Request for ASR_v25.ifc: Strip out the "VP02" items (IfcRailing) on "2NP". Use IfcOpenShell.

First a look at what the model holds.

```python
import ifcopenshell
import ifcopenshell.util.element

model = ifcopenshell.open("ASR_v25.ifc")
print(model.schema)
storey = next(s for s in model.by_type("IfcBuildingStorey") if s.Name == "2NP")
railings = [e for e in ifcopenshell.util.element.get_decomposition(storey) if e.is_a("IfcRailing")]
seen = {}
for e in railings:
    element_type = ifcopenshell.util.element.get_type(e)
    name = element_type.Name if element_type not in (None, e) else None
    seen[name] = seen.get(name, 0) + 1
for name, count in sorted(seen.items(), key=str):
    print(count, "x", name)
```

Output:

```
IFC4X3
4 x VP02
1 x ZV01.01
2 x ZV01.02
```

```python
import ifcopenshell
import ifcopenshell.api.root
import ifcopenshell.util.element

model = ifcopenshell.open("ASR_v25.ifc")

storey = next(s for s in model.by_type("IfcBuildingStorey") if s.Name == "2NP")
railings = [e for e in ifcopenshell.util.element.get_decomposition(storey) if e.is_a("IfcRailing")]
targets = [e for e in railings if (t := ifcopenshell.util.element.get_type(e)) not in (None, e) and t.Name == "VP02"]

for e in targets:
    ifcopenshell.api.root.remove_product(model, product=e)
print(len(targets), "removed")

model.write("ASR_v25_v2.ifc")
```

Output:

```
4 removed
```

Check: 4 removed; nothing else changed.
